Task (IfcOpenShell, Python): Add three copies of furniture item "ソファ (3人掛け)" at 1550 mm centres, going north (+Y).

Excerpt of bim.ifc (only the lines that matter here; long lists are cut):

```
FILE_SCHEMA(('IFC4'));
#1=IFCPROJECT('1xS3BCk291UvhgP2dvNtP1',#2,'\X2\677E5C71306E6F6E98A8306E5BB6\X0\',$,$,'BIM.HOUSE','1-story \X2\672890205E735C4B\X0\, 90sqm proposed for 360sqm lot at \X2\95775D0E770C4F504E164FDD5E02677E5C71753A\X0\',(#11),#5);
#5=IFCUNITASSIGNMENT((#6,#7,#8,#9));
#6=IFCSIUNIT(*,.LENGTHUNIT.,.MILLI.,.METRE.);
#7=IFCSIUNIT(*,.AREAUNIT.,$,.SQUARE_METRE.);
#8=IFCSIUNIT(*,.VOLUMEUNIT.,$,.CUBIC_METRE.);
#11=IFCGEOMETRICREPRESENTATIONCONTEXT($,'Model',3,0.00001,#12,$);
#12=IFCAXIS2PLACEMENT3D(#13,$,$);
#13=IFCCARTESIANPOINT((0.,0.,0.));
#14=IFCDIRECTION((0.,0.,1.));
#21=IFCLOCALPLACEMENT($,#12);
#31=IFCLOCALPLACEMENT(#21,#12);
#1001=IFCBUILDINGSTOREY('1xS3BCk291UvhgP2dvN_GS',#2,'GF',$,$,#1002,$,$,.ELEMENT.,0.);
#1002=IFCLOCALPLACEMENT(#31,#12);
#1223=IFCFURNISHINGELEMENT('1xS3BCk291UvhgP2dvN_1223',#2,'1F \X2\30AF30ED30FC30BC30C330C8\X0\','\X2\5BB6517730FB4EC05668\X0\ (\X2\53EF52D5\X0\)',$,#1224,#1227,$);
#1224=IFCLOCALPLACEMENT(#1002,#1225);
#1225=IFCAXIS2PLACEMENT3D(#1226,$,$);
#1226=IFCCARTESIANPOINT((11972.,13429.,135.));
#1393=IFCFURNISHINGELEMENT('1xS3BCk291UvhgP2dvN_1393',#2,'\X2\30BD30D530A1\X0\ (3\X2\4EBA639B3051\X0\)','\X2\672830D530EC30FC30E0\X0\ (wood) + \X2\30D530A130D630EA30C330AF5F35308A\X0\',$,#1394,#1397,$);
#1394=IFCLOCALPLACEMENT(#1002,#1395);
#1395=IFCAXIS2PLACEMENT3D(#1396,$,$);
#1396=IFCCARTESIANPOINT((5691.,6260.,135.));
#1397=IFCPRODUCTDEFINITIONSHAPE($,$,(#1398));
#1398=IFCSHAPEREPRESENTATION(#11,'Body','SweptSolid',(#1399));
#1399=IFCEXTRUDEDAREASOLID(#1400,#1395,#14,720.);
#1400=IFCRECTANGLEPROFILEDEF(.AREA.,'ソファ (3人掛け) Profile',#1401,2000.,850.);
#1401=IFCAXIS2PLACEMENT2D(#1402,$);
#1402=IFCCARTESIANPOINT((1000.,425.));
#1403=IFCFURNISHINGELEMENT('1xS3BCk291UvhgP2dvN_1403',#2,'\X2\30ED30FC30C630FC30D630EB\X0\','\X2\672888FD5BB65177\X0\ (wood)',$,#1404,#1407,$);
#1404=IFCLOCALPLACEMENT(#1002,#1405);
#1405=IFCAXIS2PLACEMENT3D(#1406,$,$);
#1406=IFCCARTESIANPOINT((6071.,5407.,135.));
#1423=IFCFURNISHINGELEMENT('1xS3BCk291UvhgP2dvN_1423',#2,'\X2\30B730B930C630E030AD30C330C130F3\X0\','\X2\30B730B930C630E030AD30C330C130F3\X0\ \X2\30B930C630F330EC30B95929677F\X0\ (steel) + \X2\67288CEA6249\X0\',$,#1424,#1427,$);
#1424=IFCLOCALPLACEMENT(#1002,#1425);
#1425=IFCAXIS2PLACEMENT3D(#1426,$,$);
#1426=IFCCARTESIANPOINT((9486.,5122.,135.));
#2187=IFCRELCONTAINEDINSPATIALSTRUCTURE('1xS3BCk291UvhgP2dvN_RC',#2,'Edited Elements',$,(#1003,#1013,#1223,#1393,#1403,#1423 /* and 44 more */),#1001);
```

```python
import numpy as np
import ifcopenshell
import ifcopenshell.api.geometry
import ifcopenshell.api.root
import ifcopenshell.util.element
import ifcopenshell.util.placement

model = ifcopenshell.open("bim.ifc")


def reuse_history(source, copy):
    """copy_class also copies each property set's owner history, people and application; keep the originals."""
    for rel in copy.IsDefinedBy:
        if rel.is_a("IfcRelDefinesByProperties") and (history := rel.RelatingPropertyDefinition.OwnerHistory):
            rel.RelatingPropertyDefinition.OwnerHistory = source.OwnerHistory
            ifcopenshell.util.element.remove_deep2(model, history)


source = model.by_guid("1xS3BCk291UvhgP2dvN_1393")
base = ifcopenshell.util.placement.get_local_placement(source.ObjectPlacement)
step = np.array([0.0, 1.0, 0.0]) * 1550.0

for i in range(1, 4):
    copy = ifcopenshell.api.root.copy_class(model, product=source)
    copy.Representation = ifcopenshell.util.element.copy_deep(
        model, source.Representation, exclude=["IfcGeometricRepresentationContext", "IfcRepresentationMap"]
    )
    reuse_history(source, copy)
    matrix = base.copy()
    matrix[:3, 3] += i * step
    print("added at", matrix[:3, 3].round(3) + 0.0)
    ifcopenshell.api.geometry.edit_object_placement(model, product=copy, matrix=matrix, is_si=False)

model.write("bim_edited.ifc")
```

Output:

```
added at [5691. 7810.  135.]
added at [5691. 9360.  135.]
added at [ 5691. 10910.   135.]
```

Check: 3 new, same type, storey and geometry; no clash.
